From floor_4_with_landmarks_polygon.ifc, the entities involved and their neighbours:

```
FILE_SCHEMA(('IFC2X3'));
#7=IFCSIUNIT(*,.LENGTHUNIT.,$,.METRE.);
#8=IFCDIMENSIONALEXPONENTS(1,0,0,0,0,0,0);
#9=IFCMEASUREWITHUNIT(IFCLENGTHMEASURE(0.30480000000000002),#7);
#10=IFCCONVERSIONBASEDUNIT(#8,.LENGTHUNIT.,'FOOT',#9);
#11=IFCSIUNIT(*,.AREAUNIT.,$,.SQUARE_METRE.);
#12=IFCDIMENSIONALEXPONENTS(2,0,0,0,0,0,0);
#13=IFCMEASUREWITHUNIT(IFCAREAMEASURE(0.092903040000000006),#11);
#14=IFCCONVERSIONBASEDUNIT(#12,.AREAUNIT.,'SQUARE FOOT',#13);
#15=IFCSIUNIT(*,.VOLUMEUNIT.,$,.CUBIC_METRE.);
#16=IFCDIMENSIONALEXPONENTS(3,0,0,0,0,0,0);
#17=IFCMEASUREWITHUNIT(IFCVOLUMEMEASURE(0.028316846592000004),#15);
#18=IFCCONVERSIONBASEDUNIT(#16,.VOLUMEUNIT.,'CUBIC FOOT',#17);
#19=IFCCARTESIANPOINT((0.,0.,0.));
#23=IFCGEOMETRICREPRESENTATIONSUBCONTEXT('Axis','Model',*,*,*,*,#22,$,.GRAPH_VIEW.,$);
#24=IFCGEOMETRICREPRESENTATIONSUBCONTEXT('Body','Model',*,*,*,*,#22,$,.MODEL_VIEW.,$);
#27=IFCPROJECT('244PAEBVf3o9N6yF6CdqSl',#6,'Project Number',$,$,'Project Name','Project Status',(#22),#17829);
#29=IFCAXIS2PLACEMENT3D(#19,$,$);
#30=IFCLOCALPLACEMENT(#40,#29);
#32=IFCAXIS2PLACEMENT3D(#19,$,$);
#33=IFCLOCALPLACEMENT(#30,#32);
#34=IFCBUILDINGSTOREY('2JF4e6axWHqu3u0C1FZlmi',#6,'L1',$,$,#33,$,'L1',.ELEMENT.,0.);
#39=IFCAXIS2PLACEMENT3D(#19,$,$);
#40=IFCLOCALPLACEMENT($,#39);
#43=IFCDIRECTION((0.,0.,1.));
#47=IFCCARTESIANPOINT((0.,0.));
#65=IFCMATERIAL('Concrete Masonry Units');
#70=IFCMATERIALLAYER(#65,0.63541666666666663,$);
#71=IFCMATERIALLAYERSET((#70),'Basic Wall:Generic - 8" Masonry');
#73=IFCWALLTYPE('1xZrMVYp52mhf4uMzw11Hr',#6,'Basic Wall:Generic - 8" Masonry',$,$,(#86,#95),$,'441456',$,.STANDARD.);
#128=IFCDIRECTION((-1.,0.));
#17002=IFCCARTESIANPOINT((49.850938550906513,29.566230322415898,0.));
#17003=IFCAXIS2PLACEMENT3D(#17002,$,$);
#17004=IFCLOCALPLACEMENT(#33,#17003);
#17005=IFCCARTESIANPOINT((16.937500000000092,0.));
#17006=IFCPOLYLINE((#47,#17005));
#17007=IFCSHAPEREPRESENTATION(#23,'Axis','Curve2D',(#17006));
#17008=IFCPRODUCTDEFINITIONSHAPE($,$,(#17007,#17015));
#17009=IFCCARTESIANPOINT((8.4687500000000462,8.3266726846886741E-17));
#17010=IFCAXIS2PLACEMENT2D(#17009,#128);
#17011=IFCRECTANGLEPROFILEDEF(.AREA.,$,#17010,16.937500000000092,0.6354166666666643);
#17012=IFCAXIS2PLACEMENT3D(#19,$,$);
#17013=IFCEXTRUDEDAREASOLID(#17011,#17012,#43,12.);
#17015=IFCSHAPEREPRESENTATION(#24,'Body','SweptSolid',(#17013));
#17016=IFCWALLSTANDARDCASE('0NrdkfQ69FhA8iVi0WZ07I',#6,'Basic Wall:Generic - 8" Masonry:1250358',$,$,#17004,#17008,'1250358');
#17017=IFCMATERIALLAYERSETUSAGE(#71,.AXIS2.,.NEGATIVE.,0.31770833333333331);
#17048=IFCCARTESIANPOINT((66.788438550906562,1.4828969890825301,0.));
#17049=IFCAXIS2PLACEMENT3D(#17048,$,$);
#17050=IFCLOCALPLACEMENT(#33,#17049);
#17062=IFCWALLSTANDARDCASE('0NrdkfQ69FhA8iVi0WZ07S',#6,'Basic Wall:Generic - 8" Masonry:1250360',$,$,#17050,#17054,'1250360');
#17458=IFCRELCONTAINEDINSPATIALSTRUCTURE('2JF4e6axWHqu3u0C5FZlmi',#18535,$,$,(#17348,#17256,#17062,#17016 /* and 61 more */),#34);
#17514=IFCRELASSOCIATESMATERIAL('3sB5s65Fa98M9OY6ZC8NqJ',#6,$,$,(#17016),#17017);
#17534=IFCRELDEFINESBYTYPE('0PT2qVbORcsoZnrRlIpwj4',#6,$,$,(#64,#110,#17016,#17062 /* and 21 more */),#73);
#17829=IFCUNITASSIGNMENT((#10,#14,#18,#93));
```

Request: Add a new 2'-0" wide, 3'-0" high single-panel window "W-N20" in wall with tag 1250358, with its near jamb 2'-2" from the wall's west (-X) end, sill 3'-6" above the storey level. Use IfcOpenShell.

```python
import numpy as np
import ifcopenshell
import ifcopenshell.api.feature
import ifcopenshell.api.geometry
import ifcopenshell.api.root
import ifcopenshell.api.spatial
import ifcopenshell.api.type
import ifcopenshell.geom
import ifcopenshell.util.element
import ifcopenshell.util.placement
import ifcopenshell.util.representation
import ifcopenshell.util.shape
import ifcopenshell.util.unit

model = ifcopenshell.open("floor_4_with_landmarks_polygon.ifc")
unit_scale = ifcopenshell.util.unit.calculate_unit_scale(model)
settings = ifcopenshell.geom.settings()


def volume(element):
    """Net volume in cubic metres, openings subtracted."""
    shape = ifcopenshell.geom.create_shape(settings, element)
    return ifcopenshell.util.shape.get_volume(shape.geometry)


wall = model.by_id(17016)
storey = ifcopenshell.util.element.get_container(wall, ifc_class="IfcBuildingStorey")
context = ifcopenshell.util.representation.get_context(model, "Model", "Body", "MODEL_VIEW")
before = volume(wall)

width, height, from_end, sill = 0.6096, 0.9144, 0.6604, 1.0668  # metres

# The wall runs along its own X axis, and the end named is its -X end.
wall_shape = ifcopenshell.geom.create_shape(settings, wall)
x, y, z = ifcopenshell.util.shape.get_vertices(wall_shape.geometry).T
start = x.min() + from_end
face, thickness = float(y.min()), float(y.max() - y.min())
wall_matrix = ifcopenshell.util.placement.get_local_placement(wall.ObjectPlacement)
level = ifcopenshell.util.placement.get_local_placement(storey.ObjectPlacement)[2, 3]


def in_wall(x, y):
    """Placement at x, y metres in the wall's axes, at sill height."""
    matrix = wall_matrix.copy()
    matrix[:, 3] = wall_matrix @ np.array([x / unit_scale, y / unit_scale, 0.0, 1.0])
    matrix[2, 3] = level + sill / unit_scale
    return matrix


# Opening: a box that overshoots both wall faces by 50 mm.
opening = ifcopenshell.api.root.create_entity(model, ifc_class="IfcOpeningElement")
box = ifcopenshell.api.geometry.add_wall_representation(
    model, context=context, length=width, height=height, thickness=thickness + 0.1
)
ifcopenshell.api.geometry.assign_representation(model, product=opening, representation=box)
ifcopenshell.api.geometry.edit_object_placement(model, product=opening, matrix=in_wall(start, face - 0.05), is_si=False)
ifcopenshell.api.feature.add_feature(model, feature=opening, element=wall)

window = ifcopenshell.api.root.create_entity(model, ifc_class="IfcWindow", name="W-N20")
window.OverallWidth, window.OverallHeight = width / unit_scale, height / unit_scale
body = ifcopenshell.api.geometry.add_window_representation(
    model,
    context=context,
    overall_width=window.OverallWidth,
    overall_height=window.OverallHeight,
    partition_type="SINGLE_PANEL",
)
ifcopenshell.api.geometry.assign_representation(model, product=window, representation=body)
ifcopenshell.api.spatial.assign_container(model, products=[window], relating_structure=storey)
fills = ifcopenshell.api.feature.add_filling(model, opening=opening, element=window)
fills.OwnerHistory = window.OwnerHistory  # required in IFC2X3

# IFC2X3 keeps the operation on the window style.
style = ifcopenshell.api.root.create_entity(model, ifc_class="IfcWindowStyle", name="W-N20")
style.OperationType, style.ConstructionType = "SINGLE_PANEL", "NOTDEFINED"
style.ParameterTakesPrecedence = style.Sizeable = False
ifcopenshell.api.type.assign_type(model, related_objects=[window], relating_type=style)

# Centre the window in the wall's thickness.
ifcopenshell.api.geometry.edit_object_placement(model, product=window, matrix=in_wall(start, face), is_si=False)
window_shape = ifcopenshell.geom.create_shape(settings, window)
depth = ifcopenshell.util.shape.get_vertices(window_shape.geometry)[:, 1]
offset = face + thickness / 2 - (depth.min() + depth.max()) / 2
ifcopenshell.api.geometry.edit_object_placement(model, product=window, matrix=in_wall(start, offset), is_si=False)

after = volume(wall)

print(f"wall volume {before:.3f} -> {after:.3f} m3")

model.write("floor_4_with_landmarks_polygon_rev.ifc")
```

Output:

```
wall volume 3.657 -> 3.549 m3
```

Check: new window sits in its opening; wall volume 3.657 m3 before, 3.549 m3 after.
